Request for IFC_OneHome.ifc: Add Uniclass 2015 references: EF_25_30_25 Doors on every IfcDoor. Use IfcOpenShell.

First a look at what the model holds.

```python
import ifcopenshell

model = ifcopenshell.open("IFC_OneHome.ifc")
print(model.schema)
print("classifications:", [c.Name for c in model.by_type("IfcClassification")])
for ifc_class in ("IfcDoor", "IfcRoof", "IfcStair", "IfcWall", "IfcWindow"):
    print(ifc_class, len(model.by_type(ifc_class)))
```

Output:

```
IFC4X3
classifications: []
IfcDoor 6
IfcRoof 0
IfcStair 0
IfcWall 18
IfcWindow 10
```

```python
import ifcopenshell
import ifcopenshell.api.classification

model = ifcopenshell.open("IFC_OneHome.ifc")

system = ifcopenshell.api.classification.add_classification(model, classification="Uniclass 2015")

codes = {
    "IfcDoor": ("EF_25_30_25", "Doors"),
}
for ifc_class, (code, name) in codes.items():
    products = model.by_type(ifc_class)
    ifcopenshell.api.classification.add_reference(
        model, products=products, classification=system, identification=code, name=name
    )
    print(code, len(products))

model.write("IFC_OneHome_v2.ifc")
```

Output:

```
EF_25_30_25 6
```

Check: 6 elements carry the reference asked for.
